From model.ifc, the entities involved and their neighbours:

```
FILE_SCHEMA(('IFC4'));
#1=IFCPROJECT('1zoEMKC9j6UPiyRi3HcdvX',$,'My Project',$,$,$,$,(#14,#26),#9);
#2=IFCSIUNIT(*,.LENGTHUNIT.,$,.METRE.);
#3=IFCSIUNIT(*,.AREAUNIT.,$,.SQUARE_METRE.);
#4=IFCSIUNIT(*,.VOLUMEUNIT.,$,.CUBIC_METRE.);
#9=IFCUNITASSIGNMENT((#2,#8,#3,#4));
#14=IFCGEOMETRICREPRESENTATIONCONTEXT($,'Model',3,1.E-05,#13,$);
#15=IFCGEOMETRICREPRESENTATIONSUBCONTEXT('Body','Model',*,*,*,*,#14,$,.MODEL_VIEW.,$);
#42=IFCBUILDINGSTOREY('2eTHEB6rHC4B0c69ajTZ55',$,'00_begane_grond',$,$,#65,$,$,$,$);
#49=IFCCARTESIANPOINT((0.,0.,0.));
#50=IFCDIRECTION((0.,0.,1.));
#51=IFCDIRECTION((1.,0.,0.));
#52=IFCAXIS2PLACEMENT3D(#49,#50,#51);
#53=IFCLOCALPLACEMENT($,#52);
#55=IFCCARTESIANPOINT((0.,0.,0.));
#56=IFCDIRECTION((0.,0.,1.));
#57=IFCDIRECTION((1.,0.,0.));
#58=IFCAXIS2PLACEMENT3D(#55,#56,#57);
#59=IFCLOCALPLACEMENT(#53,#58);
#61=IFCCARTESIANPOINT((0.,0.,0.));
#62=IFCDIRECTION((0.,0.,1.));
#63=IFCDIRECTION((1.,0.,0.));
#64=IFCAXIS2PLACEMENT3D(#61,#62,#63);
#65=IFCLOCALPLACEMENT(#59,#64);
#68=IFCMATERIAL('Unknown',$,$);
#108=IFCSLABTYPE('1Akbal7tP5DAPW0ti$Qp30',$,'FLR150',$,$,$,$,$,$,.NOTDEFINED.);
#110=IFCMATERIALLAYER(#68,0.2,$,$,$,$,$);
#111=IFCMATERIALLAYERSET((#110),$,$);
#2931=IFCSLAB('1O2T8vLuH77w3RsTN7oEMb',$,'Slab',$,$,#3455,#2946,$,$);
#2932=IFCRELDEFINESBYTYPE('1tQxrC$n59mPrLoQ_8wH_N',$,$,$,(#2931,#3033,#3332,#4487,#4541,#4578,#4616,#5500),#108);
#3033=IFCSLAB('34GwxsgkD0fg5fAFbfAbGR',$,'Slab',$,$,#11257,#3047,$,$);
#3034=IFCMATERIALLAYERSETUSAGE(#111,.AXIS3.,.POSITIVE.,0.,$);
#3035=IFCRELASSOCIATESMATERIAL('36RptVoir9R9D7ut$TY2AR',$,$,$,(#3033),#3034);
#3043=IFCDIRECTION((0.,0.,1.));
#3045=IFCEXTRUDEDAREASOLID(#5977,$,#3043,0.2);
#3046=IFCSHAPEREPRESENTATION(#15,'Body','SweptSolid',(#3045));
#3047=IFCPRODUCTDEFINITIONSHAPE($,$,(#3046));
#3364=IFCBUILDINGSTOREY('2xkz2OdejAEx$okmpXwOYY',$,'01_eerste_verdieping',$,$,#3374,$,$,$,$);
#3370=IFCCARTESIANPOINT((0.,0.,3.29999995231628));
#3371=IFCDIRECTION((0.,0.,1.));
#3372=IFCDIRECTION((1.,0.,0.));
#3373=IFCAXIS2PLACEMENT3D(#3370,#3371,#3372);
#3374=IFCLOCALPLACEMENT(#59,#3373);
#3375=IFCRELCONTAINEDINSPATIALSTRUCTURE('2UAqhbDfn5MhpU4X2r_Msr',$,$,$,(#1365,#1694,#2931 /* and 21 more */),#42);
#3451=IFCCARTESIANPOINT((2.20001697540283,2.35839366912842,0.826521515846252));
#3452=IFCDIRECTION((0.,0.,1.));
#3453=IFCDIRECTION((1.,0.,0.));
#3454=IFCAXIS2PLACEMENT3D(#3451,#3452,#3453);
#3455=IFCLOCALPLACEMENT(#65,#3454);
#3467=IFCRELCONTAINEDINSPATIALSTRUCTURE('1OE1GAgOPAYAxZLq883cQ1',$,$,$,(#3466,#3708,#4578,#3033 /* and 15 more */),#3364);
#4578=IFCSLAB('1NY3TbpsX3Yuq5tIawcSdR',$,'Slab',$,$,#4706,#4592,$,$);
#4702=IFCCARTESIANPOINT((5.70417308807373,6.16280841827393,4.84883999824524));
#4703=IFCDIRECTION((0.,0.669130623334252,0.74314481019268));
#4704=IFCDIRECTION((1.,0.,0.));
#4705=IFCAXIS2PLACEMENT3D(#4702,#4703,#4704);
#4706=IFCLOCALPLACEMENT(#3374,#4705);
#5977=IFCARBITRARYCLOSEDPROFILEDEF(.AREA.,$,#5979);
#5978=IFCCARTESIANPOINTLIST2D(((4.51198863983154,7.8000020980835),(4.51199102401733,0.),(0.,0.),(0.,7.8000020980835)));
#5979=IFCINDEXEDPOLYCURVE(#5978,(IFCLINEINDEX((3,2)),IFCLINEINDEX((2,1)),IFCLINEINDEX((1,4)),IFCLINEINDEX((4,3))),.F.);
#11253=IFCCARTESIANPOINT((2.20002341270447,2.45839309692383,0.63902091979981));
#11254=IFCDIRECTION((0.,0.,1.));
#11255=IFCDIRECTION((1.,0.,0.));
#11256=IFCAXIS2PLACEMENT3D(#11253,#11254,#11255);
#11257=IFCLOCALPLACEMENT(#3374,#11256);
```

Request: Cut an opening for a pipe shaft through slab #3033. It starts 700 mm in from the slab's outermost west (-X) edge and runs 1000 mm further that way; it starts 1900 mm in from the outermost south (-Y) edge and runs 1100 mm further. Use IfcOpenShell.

```python
import numpy as np
import ifcopenshell
import ifcopenshell.api.feature
import ifcopenshell.api.geometry
import ifcopenshell.api.root
import ifcopenshell.geom
import ifcopenshell.util.placement
import ifcopenshell.util.representation
import ifcopenshell.util.shape
import ifcopenshell.util.unit

model = ifcopenshell.open("model.ifc")
unit_scale = ifcopenshell.util.unit.calculate_unit_scale(model)
settings = ifcopenshell.geom.settings()


def volume(element):
    """Net volume in cubic metres, openings subtracted."""
    shape = ifcopenshell.geom.create_shape(settings, element)
    return ifcopenshell.util.shape.get_volume(shape.geometry)


slab = model.by_id(3033)
before = volume(slab)

# Extent in the slab's own axes, in metres. The edges named are its -X and -Y sides.
slab_shape = ifcopenshell.geom.create_shape(settings, slab)
vertices = ifcopenshell.util.shape.get_vertices(slab_shape.geometry)
x_min, y_min, bottom = vertices.min(axis=0)
top = vertices[:, 2].max()

opening = ifcopenshell.api.root.create_entity(model, ifc_class="IfcOpeningElement", name="Pipe shaft opening", predefined_type="OPENING")
context = ifcopenshell.util.representation.get_context(model, "Model", "Body", "MODEL_VIEW")
width, depth = 1, 1.1
outline = [(0.0, 0.0), (width, 0.0), (width, depth), (0.0, depth), (0.0, 0.0)]
# Overshoot both faces by 50 mm so the cut is clean.
shape = ifcopenshell.api.geometry.add_slab_representation(
    model, context=context, depth=top - bottom + 0.1, polyline=outline
)
ifcopenshell.api.geometry.assign_representation(model, product=opening, representation=shape)

matrix = ifcopenshell.util.placement.get_local_placement(slab.ObjectPlacement)
matrix[:, 3] = matrix @ np.append(np.array([x_min + 0.7, y_min + 1.9, bottom - 0.05]) / unit_scale, 1.0)
ifcopenshell.api.geometry.edit_object_placement(model, product=opening, matrix=matrix, is_si=False)
ifcopenshell.api.feature.add_feature(model, feature=opening, element=slab)

after = volume(slab)

print(f"slab volume {before:.3f} -> {after:.3f} m3")

model.write("model-out.ifc")
```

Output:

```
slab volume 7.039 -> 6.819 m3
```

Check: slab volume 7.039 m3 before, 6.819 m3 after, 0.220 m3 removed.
